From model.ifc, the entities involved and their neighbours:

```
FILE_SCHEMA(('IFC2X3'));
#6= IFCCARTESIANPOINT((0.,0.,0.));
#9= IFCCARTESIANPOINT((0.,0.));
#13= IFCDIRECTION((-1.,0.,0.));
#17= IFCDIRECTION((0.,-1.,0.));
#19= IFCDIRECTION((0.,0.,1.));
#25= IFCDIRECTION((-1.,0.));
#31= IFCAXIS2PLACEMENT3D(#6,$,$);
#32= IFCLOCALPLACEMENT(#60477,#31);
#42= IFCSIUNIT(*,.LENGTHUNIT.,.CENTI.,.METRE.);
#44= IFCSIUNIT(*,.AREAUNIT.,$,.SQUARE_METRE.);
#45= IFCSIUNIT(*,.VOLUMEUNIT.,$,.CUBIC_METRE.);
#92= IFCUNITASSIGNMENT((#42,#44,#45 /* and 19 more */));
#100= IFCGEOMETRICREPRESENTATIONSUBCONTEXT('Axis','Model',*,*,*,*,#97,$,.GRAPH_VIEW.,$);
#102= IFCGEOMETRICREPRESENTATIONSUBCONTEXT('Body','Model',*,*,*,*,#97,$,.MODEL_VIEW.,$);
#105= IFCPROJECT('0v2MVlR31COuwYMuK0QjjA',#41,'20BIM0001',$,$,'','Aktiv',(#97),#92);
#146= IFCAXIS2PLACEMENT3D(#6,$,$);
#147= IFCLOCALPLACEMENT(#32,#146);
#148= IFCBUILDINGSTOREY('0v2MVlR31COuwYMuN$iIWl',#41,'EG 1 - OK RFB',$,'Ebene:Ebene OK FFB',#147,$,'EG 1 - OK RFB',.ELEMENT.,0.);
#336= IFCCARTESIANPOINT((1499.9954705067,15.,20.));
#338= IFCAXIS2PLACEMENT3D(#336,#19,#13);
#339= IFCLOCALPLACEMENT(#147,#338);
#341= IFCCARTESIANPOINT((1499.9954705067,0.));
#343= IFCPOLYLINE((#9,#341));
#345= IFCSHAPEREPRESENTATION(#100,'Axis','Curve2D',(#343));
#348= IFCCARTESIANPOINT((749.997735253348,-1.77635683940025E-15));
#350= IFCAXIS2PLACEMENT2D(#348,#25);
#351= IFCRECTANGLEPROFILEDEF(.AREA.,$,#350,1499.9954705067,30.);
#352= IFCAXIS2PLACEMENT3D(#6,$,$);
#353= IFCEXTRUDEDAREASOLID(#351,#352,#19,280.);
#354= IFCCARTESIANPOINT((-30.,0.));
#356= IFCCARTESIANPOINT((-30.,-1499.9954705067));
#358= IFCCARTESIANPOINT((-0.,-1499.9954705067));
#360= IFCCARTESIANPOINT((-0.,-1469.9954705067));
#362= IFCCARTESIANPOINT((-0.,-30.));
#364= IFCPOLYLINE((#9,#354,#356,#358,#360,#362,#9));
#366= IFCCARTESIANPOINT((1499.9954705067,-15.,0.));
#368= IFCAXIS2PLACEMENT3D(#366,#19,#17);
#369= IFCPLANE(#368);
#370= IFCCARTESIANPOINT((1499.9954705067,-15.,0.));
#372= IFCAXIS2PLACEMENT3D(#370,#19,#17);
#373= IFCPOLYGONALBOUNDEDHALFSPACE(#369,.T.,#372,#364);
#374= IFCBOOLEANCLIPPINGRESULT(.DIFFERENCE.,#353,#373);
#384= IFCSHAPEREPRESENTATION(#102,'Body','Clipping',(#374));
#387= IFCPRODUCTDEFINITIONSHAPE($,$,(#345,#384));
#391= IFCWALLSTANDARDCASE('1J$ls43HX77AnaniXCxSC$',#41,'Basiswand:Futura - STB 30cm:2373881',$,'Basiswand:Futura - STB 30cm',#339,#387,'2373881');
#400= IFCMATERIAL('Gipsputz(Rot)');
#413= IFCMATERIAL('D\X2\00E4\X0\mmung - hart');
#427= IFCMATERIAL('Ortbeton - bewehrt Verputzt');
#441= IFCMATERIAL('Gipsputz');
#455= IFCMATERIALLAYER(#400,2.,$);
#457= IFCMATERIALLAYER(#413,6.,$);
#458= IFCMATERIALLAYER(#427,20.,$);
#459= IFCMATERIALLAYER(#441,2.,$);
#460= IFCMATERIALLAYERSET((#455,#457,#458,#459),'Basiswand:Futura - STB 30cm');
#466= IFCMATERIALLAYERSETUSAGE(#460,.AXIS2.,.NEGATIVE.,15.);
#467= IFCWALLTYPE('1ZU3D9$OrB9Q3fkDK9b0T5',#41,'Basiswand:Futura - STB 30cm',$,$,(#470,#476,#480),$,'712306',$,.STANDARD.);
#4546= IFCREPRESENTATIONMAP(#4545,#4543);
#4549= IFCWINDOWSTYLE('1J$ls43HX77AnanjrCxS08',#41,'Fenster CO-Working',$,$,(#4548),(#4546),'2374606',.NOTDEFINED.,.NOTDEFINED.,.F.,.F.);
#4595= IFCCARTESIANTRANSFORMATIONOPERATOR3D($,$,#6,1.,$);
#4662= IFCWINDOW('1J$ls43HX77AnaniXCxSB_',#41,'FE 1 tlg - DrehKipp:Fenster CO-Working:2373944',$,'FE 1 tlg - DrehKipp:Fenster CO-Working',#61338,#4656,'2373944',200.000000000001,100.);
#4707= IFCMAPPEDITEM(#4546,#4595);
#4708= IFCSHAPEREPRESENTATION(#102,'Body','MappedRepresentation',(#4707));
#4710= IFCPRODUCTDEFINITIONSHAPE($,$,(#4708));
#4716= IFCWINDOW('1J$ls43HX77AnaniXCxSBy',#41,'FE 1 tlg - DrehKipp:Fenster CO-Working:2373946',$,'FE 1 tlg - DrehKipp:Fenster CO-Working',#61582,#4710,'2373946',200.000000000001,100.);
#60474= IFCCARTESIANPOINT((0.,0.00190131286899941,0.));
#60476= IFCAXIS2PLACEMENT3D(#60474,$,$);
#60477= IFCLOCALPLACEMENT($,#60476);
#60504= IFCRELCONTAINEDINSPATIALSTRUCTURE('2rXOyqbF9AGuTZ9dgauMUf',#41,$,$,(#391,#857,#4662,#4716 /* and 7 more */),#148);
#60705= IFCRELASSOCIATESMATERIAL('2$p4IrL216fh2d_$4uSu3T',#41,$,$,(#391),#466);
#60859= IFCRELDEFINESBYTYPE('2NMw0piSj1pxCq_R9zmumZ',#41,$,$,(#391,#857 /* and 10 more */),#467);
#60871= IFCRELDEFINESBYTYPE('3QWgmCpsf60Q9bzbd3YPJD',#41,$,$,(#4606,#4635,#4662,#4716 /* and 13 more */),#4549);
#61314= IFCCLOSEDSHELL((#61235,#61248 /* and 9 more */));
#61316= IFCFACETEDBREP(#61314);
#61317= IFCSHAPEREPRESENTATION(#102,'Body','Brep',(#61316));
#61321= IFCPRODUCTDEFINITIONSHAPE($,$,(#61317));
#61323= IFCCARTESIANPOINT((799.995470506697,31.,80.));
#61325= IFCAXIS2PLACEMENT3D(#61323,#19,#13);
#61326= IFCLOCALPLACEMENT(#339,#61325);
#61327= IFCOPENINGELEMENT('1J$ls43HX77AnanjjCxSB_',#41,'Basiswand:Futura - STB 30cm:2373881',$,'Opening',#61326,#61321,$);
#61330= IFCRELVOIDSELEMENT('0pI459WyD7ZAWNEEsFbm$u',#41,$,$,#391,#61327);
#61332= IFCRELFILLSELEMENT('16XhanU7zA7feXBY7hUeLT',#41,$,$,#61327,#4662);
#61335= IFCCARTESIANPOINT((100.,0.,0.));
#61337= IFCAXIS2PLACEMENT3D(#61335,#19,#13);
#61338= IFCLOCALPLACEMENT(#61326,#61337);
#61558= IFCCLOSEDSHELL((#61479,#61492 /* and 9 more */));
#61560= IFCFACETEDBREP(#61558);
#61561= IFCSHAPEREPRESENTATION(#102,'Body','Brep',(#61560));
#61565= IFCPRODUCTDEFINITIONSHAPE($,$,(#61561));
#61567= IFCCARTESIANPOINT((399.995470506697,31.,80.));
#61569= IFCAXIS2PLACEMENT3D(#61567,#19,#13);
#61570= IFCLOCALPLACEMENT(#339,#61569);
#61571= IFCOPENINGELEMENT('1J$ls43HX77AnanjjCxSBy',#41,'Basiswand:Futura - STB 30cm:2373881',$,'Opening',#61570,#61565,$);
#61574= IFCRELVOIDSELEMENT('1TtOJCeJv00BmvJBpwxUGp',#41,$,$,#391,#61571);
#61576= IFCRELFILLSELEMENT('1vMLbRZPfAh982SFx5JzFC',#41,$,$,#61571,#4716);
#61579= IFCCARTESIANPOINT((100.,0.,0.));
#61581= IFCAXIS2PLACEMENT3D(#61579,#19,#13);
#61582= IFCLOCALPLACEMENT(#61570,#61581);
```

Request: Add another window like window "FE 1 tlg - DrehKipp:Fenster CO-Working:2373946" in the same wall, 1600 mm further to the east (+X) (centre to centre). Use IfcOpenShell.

```python
import ifcopenshell
import ifcopenshell.api.feature
import ifcopenshell.api.geometry
import ifcopenshell.api.root
import ifcopenshell.geom
import ifcopenshell.util.element
import ifcopenshell.util.placement
import ifcopenshell.util.shape
import ifcopenshell.util.unit

model = ifcopenshell.open("model.ifc")
unit_scale = ifcopenshell.util.unit.calculate_unit_scale(model)
settings = ifcopenshell.geom.settings()


def volume(element):
    """Net volume in cubic metres, openings subtracted."""
    shape = ifcopenshell.geom.create_shape(settings, element)
    return ifcopenshell.util.shape.get_volume(shape.geometry)


def reuse_history(source, copy):
    """copy_class also copies each property set's owner history, people and application; keep the originals."""
    for rel in copy.IsDefinedBy:
        if rel.is_a("IfcRelDefinesByProperties") and (history := rel.RelatingPropertyDefinition.OwnerHistory):
            rel.RelatingPropertyDefinition.OwnerHistory = source.OwnerHistory
            ifcopenshell.util.element.remove_deep2(model, history)


window = model.by_id(4716)
opening = window.FillsVoids[0].RelatingOpeningElement
wall = opening.VoidsElements[0].RelatingBuildingElement
before = volume(wall)
shift = ifcopenshell.util.placement.get_local_placement(wall.ObjectPlacement)[:3, 0] * -1.6 / unit_scale

# copy_class copies the void relationship, type, container and properties, but no geometry.
new_opening = ifcopenshell.api.root.copy_class(model, product=opening)
new_opening.Representation = ifcopenshell.util.element.copy_deep(
    model, opening.Representation, exclude=["IfcGeometricRepresentationContext", "IfcRepresentationMap"]
)
new_opening.Name = "Basiswand:Futura - STB 30cm"
new_window = ifcopenshell.api.root.copy_class(model, product=window)
new_window.Representation = ifcopenshell.util.element.copy_deep(
    model, window.Representation, exclude=["IfcGeometricRepresentationContext", "IfcRepresentationMap"]
)
new_window.Name = "FE 1 tlg - DrehKipp:Fenster CO-Working"
new_window.Tag = None
reuse_history(window, new_window)
fills = ifcopenshell.api.feature.add_filling(model, opening=new_opening, element=new_window)
fills.OwnerHistory = new_window.OwnerHistory  # required in IFC2X3

for old, new in ((opening, new_opening), (window, new_window)):
    matrix = ifcopenshell.util.placement.get_local_placement(old.ObjectPlacement)
    matrix[:3, 3] += shift
    ifcopenshell.api.geometry.edit_object_placement(model, product=new, matrix=matrix, is_si=False)

after = volume(wall)

print(f"wall volume {before:.3f} -> {after:.3f} m3")

model.write("model_rev.ifc")
```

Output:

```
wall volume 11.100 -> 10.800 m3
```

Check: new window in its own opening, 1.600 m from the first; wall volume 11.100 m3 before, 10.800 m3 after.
